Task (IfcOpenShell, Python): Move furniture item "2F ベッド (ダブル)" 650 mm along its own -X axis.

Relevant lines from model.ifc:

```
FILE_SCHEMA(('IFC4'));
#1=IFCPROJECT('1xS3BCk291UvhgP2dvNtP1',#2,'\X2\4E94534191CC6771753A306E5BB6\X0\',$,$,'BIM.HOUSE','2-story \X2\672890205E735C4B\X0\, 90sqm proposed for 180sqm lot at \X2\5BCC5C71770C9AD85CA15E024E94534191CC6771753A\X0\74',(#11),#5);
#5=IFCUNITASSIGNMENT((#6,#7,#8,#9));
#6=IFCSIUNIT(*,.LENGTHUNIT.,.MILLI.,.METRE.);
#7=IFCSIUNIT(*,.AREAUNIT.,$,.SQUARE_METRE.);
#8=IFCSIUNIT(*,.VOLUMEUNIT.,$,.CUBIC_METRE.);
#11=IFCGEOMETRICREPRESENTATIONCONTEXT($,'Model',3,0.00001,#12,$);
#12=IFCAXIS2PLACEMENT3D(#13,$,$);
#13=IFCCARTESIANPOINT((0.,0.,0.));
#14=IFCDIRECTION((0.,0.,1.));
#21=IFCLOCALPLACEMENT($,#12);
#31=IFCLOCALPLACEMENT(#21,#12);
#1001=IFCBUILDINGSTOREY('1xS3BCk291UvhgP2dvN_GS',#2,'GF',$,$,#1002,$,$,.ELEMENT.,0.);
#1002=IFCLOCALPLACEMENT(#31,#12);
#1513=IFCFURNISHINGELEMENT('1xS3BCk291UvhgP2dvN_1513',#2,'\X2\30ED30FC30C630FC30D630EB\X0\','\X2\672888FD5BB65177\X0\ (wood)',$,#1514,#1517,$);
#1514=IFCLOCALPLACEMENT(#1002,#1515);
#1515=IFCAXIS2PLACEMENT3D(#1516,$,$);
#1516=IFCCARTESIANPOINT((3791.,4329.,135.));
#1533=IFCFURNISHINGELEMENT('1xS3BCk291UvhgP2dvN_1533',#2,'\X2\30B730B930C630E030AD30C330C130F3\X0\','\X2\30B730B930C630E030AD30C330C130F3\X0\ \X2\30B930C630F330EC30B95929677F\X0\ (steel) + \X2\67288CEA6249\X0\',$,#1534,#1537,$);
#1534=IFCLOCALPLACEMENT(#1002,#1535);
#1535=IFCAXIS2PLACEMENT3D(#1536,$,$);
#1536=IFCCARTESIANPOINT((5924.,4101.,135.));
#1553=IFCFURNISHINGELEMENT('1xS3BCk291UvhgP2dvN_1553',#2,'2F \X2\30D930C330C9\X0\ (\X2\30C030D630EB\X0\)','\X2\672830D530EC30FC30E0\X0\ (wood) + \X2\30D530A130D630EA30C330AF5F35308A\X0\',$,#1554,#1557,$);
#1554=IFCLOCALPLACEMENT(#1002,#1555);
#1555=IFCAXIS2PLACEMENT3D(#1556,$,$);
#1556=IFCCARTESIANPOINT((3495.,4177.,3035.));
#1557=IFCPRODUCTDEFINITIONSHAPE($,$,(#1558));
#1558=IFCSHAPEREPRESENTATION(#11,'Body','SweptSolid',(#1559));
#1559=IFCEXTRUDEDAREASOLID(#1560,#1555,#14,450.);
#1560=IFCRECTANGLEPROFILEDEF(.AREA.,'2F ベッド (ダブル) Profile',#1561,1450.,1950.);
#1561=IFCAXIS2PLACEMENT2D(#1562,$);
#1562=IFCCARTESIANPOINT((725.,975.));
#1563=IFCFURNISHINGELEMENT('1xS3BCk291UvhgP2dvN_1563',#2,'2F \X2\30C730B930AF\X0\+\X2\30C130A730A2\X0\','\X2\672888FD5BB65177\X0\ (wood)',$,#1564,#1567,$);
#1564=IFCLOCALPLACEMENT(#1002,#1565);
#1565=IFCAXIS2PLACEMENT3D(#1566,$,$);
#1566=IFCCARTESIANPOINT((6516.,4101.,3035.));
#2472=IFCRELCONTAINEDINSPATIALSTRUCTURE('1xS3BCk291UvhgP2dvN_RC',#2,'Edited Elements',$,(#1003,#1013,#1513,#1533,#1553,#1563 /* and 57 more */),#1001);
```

```python
import ifcopenshell
import ifcopenshell.api.geometry
import ifcopenshell.util.placement
import ifcopenshell.util.unit

model = ifcopenshell.open("model.ifc")
unit_scale = ifcopenshell.util.unit.calculate_unit_scale(model)

item = model.by_guid("1xS3BCk291UvhgP2dvN_1553")
matrix = ifcopenshell.util.placement.get_local_placement(item.ObjectPlacement)
matrix[:3, 3] -= matrix[:3, 0] * 0.65 / unit_scale
ifcopenshell.api.geometry.edit_object_placement(model, product=item, matrix=matrix, is_si=False)

print(ifcopenshell.util.placement.get_local_placement(item.ObjectPlacement).round(3) + 0.0)

model.write("model-out.ifc")
```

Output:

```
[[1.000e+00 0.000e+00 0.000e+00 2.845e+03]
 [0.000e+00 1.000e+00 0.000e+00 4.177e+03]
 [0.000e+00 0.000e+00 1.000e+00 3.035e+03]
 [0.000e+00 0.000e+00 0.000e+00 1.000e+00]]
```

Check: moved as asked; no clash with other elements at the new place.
